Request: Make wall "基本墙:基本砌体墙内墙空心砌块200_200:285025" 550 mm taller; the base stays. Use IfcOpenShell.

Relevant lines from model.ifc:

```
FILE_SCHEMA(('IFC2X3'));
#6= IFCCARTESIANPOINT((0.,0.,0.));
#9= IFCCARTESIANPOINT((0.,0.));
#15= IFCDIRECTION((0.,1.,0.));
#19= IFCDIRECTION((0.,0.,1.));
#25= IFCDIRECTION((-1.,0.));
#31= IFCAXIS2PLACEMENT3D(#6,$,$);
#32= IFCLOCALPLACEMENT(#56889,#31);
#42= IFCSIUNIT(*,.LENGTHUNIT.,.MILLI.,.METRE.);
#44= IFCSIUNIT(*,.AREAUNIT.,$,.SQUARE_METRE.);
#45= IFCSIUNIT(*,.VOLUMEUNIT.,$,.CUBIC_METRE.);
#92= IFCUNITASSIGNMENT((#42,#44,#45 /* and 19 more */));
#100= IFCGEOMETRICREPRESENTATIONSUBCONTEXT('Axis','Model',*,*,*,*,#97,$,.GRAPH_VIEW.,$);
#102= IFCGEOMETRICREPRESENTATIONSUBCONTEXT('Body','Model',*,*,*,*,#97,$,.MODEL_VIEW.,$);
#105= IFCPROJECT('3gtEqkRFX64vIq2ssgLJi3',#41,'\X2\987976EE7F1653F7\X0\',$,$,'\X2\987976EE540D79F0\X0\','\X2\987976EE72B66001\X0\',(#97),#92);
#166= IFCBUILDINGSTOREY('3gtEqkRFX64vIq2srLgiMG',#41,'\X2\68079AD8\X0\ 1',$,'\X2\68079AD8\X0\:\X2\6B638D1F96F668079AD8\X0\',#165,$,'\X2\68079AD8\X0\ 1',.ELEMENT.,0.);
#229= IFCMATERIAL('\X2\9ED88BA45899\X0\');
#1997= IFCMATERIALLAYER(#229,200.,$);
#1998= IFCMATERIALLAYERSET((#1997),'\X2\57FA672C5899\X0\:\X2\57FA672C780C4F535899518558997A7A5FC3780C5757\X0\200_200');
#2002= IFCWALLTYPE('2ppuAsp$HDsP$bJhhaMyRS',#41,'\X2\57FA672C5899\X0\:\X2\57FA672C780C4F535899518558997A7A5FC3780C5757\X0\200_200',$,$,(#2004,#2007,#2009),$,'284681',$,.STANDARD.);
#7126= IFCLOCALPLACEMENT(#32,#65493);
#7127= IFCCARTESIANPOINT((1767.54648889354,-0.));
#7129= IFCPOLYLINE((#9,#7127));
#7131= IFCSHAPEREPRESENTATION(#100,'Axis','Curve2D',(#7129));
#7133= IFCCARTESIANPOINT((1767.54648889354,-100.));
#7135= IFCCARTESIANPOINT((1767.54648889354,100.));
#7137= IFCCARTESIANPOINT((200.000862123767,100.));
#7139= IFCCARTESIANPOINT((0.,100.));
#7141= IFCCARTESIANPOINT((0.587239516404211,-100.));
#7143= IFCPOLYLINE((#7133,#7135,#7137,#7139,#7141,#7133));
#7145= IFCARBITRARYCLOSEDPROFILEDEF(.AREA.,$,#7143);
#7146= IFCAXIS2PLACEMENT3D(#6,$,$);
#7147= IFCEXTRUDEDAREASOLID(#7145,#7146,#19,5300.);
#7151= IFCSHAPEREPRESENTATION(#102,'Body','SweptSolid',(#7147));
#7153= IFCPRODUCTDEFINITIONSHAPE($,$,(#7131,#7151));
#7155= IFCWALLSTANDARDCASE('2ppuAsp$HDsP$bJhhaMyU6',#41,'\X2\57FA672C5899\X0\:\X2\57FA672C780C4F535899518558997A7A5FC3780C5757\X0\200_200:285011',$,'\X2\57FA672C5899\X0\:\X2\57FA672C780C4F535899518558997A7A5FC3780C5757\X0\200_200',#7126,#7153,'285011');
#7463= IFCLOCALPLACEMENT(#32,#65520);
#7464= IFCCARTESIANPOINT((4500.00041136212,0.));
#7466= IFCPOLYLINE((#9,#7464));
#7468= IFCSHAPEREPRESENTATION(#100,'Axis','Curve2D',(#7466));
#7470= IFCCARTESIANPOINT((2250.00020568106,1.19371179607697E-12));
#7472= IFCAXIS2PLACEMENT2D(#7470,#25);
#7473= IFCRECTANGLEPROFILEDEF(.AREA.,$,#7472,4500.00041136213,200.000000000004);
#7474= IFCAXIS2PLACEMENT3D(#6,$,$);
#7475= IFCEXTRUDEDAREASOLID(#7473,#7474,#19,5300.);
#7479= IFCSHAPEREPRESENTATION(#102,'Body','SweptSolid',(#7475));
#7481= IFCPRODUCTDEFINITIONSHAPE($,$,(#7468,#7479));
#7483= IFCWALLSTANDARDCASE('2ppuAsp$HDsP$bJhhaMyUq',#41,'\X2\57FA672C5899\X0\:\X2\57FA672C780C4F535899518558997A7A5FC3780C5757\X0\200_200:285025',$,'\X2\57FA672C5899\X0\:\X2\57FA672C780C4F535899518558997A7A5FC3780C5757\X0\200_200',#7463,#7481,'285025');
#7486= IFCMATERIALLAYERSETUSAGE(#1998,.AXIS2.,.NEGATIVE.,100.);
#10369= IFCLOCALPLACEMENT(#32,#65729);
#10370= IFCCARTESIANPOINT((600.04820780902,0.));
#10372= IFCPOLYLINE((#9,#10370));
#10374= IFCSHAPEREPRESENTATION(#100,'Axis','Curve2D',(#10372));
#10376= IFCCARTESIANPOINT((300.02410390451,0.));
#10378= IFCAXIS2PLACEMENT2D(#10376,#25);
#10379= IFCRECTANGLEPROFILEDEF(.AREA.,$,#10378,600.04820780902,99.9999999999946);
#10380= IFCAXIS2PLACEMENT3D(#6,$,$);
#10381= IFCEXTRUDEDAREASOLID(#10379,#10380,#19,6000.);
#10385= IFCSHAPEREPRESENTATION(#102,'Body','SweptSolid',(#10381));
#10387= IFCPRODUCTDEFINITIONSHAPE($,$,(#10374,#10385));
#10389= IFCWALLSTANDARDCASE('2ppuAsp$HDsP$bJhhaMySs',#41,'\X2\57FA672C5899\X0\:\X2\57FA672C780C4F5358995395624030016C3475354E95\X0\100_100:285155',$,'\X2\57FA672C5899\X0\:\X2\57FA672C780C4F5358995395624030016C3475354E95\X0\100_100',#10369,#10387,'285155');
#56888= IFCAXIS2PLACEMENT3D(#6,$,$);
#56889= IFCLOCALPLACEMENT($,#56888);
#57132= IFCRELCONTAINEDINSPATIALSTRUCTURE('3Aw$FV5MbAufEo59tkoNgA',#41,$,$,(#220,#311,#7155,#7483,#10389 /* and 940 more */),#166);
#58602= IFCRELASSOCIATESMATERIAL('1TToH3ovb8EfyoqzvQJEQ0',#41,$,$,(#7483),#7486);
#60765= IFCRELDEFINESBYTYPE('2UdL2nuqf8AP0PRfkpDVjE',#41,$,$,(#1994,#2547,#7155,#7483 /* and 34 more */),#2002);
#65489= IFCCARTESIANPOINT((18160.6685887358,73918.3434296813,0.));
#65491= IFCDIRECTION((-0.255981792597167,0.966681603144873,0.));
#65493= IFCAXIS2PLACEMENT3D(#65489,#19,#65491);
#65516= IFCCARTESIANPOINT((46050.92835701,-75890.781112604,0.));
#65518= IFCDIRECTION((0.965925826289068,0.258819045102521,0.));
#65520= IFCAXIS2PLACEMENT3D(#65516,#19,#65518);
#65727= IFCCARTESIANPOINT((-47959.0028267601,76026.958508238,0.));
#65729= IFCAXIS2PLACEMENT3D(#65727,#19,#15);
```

```python
import ifcopenshell
import ifcopenshell.geom
import ifcopenshell.util.representation
import ifcopenshell.util.shape

model = ifcopenshell.open("model.ifc")
settings = ifcopenshell.geom.settings()


def volume(element):
    """Net volume in cubic metres, openings subtracted."""
    shape = ifcopenshell.geom.create_shape(settings, element)
    return ifcopenshell.util.shape.get_volume(shape.geometry)


wall = model.by_guid("2ppuAsp$HDsP$bJhhaMyUq")
before = volume(wall)

body = ifcopenshell.util.representation.get_representation(wall, "Model", "Body")
solid = body.Items[0]
old_height = solid.Depth
solid.Depth += 550.0
after = volume(wall)

print(f"height {old_height:g} -> {solid.Depth:g}, volume {before:.3f} -> {after:.3f} m3")

model.write("model_v2.ifc")
```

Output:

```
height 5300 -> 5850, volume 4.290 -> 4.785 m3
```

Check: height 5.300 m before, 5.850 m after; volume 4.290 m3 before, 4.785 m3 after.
